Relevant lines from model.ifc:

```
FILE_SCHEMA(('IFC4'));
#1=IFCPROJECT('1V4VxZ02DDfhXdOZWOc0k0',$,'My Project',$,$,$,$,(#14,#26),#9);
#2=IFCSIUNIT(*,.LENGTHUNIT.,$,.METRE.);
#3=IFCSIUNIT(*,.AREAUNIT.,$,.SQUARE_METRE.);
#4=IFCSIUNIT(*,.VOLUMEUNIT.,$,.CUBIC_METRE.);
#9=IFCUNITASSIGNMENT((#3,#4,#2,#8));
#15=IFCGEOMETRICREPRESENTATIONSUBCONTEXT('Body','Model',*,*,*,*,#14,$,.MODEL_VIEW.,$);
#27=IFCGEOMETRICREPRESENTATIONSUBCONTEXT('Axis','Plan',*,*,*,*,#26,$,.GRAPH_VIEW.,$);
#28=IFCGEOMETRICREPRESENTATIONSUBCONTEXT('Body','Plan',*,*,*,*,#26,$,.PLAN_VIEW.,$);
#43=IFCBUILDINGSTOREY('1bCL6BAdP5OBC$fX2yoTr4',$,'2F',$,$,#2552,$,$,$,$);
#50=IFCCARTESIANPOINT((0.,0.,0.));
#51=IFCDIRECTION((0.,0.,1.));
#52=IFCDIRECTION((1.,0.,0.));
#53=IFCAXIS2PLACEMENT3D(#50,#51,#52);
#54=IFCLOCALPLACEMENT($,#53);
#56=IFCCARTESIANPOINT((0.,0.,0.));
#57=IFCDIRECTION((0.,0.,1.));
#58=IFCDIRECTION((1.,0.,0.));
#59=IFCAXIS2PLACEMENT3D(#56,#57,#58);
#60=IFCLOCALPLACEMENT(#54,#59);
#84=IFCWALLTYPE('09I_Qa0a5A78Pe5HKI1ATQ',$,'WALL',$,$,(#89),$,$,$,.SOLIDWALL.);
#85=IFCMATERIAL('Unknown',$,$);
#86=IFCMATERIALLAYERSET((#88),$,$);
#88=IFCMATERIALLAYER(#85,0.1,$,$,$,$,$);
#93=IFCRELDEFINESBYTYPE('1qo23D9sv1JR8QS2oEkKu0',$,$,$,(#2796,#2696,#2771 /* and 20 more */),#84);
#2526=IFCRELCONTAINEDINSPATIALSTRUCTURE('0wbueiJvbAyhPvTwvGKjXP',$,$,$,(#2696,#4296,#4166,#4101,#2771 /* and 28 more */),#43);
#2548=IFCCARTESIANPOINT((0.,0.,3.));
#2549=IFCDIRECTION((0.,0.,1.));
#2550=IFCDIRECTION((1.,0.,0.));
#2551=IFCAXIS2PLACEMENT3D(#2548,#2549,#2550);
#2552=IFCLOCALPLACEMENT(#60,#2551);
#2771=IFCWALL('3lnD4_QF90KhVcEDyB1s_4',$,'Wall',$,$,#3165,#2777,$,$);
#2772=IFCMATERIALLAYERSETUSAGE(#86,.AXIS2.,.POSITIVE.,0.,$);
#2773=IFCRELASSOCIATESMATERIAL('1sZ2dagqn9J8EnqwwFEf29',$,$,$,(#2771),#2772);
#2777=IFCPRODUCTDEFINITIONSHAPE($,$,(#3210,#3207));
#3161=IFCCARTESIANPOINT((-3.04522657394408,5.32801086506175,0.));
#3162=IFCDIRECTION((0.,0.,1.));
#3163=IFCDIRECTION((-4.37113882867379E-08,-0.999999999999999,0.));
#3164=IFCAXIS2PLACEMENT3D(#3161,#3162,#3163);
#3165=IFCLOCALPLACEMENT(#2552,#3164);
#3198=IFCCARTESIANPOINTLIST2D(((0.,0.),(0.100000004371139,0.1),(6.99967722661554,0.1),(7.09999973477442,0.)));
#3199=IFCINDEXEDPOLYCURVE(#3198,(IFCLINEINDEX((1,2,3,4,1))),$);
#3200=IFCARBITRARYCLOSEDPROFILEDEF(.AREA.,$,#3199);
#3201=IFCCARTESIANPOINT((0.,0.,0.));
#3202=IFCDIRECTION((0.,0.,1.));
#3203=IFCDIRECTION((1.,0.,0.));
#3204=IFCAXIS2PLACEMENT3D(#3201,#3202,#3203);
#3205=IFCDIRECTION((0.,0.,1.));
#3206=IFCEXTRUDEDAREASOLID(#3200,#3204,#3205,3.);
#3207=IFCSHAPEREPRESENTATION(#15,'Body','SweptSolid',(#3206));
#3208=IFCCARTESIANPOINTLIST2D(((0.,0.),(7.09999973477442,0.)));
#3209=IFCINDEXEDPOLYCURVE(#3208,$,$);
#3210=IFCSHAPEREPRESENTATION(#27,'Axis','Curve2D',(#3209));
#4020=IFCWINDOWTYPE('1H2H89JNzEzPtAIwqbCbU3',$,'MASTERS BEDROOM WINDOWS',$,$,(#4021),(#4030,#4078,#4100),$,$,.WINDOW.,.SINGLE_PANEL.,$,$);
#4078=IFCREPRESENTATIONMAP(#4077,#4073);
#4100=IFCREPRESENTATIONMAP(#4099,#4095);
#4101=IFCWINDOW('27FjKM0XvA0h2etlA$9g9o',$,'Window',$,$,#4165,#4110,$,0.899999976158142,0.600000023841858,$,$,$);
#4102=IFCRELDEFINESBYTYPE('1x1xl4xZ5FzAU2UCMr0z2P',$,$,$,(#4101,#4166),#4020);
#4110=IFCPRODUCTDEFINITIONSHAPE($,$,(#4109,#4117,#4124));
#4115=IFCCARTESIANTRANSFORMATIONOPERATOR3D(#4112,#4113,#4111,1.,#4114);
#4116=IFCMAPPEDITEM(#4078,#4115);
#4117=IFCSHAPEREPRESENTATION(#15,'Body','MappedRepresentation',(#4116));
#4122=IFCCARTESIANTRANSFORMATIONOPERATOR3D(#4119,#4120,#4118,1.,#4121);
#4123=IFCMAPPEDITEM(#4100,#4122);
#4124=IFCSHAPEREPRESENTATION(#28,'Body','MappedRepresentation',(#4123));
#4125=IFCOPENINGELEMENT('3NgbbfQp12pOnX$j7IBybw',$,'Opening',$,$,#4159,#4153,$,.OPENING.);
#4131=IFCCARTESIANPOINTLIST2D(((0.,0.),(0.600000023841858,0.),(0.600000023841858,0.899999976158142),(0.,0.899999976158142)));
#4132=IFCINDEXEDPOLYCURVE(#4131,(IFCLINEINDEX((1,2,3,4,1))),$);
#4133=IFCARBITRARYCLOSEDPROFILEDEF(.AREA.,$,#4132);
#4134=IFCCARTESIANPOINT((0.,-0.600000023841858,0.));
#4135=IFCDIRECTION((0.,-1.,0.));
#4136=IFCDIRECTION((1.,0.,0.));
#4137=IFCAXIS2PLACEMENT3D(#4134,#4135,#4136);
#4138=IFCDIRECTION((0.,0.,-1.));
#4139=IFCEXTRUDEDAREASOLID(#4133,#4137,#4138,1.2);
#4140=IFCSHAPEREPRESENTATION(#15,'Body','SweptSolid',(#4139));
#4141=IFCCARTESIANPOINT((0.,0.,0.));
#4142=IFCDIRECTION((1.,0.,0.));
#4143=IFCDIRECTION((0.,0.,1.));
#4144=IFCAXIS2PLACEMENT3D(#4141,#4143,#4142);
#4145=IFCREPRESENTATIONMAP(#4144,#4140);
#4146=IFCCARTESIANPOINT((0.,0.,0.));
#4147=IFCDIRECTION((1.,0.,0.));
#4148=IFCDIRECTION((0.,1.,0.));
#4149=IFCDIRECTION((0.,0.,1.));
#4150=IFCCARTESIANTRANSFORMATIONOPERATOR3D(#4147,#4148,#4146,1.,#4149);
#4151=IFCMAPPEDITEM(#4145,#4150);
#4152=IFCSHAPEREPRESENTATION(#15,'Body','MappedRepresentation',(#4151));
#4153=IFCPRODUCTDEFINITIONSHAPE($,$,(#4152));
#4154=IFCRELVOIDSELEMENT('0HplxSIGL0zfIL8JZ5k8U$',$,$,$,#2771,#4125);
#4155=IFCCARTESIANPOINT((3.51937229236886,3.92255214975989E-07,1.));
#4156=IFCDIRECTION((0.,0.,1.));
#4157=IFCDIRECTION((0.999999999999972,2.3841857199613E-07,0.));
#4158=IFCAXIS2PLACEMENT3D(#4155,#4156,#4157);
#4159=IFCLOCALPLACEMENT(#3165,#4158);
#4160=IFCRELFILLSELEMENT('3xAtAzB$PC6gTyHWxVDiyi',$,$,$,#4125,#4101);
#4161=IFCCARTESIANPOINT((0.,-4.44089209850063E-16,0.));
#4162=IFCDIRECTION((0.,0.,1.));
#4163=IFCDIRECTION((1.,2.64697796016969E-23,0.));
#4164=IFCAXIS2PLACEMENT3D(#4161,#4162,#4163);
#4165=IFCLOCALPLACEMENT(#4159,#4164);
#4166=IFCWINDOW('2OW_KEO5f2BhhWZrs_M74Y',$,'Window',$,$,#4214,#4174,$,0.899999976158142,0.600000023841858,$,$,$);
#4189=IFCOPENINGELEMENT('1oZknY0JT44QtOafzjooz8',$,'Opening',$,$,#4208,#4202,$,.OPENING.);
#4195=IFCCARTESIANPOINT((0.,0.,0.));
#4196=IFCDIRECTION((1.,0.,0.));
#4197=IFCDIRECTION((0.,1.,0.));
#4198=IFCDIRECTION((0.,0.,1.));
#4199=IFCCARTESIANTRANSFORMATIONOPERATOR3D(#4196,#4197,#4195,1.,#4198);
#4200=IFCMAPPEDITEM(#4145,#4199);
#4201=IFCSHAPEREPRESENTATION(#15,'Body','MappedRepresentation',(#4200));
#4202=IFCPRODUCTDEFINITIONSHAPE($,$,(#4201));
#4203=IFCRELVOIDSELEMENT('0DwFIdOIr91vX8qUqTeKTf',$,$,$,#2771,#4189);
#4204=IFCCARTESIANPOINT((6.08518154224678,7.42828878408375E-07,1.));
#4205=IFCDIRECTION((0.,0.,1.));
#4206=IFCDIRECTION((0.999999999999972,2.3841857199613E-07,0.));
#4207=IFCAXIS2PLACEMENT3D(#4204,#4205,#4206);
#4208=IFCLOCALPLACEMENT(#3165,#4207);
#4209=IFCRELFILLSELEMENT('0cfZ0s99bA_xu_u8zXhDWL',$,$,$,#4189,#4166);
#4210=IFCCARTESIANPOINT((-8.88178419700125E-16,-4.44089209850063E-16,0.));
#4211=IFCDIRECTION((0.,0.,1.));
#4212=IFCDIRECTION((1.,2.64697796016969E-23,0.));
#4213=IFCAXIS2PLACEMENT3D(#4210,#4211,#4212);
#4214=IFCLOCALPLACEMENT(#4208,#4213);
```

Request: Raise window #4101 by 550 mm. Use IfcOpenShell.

```python
import numpy as np
import ifcopenshell
import ifcopenshell.api.geometry
import ifcopenshell.util.placement
import ifcopenshell.util.unit

model = ifcopenshell.open("model.ifc")
unit_scale = ifcopenshell.util.unit.calculate_unit_scale(model)

window = model.by_guid("27FjKM0XvA0h2etlA$9g9o")
opening = window.FillsVoids[0].RelatingOpeningElement
dz = 0.55 / unit_scale

shift = np.array([0.0, 0.0, dz])
# The window is placed relative to its opening, so it follows when the opening moves.
matrix = ifcopenshell.util.placement.get_local_placement(opening.ObjectPlacement)
matrix[:3, 3] += shift
ifcopenshell.api.geometry.edit_object_placement(
    model, product=opening, matrix=matrix, is_si=False, should_transform_children=True
)

print(f"moved by {dz * unit_scale:+.3f} m")

model.write("model_edited.ifc")
```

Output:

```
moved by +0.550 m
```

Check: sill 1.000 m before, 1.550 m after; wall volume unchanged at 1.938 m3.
